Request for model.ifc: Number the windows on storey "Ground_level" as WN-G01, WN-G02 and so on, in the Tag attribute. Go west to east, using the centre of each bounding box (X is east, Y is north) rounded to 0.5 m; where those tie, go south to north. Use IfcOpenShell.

First a look at what the model holds.

```python
import ifcopenshell
import ifcopenshell.util.element
import ifcopenshell.util.placement

model = ifcopenshell.open("model.ifc")
print(model.schema)
storey = next(s for s in model.by_type("IfcBuildingStorey") if s.Name == "Ground_level")
windows = [e for e in ifcopenshell.util.element.get_decomposition(storey) if e.is_a("IfcWindow")]
for e in sorted(windows, key=lambda e: e.id()):
    origin = ifcopenshell.util.placement.get_local_placement(e.ObjectPlacement)[:3, 3]
    print(e.id(), e.Tag, e.Name, origin.round(2) + 0.0, sep=" | ")
```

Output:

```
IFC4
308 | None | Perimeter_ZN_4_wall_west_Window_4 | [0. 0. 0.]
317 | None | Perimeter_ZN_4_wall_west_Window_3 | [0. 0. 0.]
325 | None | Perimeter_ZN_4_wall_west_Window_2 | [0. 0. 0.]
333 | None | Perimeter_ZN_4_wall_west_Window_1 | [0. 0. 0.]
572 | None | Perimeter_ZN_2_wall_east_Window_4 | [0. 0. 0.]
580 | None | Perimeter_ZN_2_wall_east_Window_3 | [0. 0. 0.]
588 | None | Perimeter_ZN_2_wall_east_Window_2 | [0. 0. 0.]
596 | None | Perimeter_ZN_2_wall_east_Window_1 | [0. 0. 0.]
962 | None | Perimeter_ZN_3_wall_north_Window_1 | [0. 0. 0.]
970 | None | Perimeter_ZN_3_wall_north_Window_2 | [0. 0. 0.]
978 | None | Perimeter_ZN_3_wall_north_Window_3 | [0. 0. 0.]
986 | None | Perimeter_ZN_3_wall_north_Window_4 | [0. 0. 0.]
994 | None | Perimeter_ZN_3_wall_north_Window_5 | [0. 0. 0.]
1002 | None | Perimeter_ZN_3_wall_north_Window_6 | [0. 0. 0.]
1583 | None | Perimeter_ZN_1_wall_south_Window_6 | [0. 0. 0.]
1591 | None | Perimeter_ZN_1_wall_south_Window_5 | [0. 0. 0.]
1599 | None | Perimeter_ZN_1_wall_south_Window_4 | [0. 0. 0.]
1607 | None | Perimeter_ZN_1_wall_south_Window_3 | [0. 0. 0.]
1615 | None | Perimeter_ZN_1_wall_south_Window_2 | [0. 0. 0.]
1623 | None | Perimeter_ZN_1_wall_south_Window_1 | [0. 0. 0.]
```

```python
import ifcopenshell
import ifcopenshell.geom
import ifcopenshell.util.element
import ifcopenshell.util.shape

model = ifcopenshell.open("model.ifc")
settings = ifcopenshell.geom.settings()
settings.set("use-world-coords", True)


def centre(element):
    shape = ifcopenshell.geom.create_shape(settings, element)
    return ifcopenshell.util.shape.get_bbox_centroid(shape.geometry)


storey = next(s for s in model.by_type("IfcBuildingStorey") if s.Name == "Ground_level")
windows = [e for e in ifcopenshell.util.element.get_decomposition(storey) if e.is_a("IfcWindow")]

# Insertion points can sit at a corner or the storey origin, so sort by the geometry (in metres).
centres = {e: centre(e) for e in windows}
windows.sort(key=lambda e: (round(centres[e][0] / 0.5), centres[e][1]))

for i, e in enumerate(windows, start=1):
    number = f"WN-G{i:02d}"
    e.Tag = number
    print(e.id(), number)

model.write("model-out.ifc")
```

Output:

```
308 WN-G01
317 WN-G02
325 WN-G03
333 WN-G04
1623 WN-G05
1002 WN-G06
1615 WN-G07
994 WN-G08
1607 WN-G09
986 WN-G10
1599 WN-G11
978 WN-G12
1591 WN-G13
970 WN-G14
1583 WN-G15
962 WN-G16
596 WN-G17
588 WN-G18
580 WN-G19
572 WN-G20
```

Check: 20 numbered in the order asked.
